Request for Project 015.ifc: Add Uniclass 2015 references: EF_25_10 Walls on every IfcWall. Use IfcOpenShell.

First a look at what the model holds.

```python
import ifcopenshell

model = ifcopenshell.open("Project 015.ifc")
print(model.schema)
print("classifications:", [c.Name for c in model.by_type("IfcClassification")])
for ifc_class in ("IfcDoor", "IfcRoof", "IfcStair", "IfcWall", "IfcWindow"):
    print(ifc_class, len(model.by_type(ifc_class)))
```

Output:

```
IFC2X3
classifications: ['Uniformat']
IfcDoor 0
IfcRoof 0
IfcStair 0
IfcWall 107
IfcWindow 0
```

```python
import ifcopenshell
import ifcopenshell.api.classification

model = ifcopenshell.open("Project 015.ifc")

# IFC2X3 requires Source and Edition and has no link from the project to the system.
system = model.create_entity("IfcClassification", Source="NBS", Edition="2015", Name="Uniclass 2015")

codes = {
    "IfcWall": ("EF_25_10", "Walls"),
}
for ifc_class, (code, name) in codes.items():
    products = model.by_type(ifc_class)
    ifcopenshell.api.classification.add_reference(
        model, products=products, classification=system, identification=code, name=name
    )
    print(code, len(products))

model.write("Project 015_edited.ifc")
```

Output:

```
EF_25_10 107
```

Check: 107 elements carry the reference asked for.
